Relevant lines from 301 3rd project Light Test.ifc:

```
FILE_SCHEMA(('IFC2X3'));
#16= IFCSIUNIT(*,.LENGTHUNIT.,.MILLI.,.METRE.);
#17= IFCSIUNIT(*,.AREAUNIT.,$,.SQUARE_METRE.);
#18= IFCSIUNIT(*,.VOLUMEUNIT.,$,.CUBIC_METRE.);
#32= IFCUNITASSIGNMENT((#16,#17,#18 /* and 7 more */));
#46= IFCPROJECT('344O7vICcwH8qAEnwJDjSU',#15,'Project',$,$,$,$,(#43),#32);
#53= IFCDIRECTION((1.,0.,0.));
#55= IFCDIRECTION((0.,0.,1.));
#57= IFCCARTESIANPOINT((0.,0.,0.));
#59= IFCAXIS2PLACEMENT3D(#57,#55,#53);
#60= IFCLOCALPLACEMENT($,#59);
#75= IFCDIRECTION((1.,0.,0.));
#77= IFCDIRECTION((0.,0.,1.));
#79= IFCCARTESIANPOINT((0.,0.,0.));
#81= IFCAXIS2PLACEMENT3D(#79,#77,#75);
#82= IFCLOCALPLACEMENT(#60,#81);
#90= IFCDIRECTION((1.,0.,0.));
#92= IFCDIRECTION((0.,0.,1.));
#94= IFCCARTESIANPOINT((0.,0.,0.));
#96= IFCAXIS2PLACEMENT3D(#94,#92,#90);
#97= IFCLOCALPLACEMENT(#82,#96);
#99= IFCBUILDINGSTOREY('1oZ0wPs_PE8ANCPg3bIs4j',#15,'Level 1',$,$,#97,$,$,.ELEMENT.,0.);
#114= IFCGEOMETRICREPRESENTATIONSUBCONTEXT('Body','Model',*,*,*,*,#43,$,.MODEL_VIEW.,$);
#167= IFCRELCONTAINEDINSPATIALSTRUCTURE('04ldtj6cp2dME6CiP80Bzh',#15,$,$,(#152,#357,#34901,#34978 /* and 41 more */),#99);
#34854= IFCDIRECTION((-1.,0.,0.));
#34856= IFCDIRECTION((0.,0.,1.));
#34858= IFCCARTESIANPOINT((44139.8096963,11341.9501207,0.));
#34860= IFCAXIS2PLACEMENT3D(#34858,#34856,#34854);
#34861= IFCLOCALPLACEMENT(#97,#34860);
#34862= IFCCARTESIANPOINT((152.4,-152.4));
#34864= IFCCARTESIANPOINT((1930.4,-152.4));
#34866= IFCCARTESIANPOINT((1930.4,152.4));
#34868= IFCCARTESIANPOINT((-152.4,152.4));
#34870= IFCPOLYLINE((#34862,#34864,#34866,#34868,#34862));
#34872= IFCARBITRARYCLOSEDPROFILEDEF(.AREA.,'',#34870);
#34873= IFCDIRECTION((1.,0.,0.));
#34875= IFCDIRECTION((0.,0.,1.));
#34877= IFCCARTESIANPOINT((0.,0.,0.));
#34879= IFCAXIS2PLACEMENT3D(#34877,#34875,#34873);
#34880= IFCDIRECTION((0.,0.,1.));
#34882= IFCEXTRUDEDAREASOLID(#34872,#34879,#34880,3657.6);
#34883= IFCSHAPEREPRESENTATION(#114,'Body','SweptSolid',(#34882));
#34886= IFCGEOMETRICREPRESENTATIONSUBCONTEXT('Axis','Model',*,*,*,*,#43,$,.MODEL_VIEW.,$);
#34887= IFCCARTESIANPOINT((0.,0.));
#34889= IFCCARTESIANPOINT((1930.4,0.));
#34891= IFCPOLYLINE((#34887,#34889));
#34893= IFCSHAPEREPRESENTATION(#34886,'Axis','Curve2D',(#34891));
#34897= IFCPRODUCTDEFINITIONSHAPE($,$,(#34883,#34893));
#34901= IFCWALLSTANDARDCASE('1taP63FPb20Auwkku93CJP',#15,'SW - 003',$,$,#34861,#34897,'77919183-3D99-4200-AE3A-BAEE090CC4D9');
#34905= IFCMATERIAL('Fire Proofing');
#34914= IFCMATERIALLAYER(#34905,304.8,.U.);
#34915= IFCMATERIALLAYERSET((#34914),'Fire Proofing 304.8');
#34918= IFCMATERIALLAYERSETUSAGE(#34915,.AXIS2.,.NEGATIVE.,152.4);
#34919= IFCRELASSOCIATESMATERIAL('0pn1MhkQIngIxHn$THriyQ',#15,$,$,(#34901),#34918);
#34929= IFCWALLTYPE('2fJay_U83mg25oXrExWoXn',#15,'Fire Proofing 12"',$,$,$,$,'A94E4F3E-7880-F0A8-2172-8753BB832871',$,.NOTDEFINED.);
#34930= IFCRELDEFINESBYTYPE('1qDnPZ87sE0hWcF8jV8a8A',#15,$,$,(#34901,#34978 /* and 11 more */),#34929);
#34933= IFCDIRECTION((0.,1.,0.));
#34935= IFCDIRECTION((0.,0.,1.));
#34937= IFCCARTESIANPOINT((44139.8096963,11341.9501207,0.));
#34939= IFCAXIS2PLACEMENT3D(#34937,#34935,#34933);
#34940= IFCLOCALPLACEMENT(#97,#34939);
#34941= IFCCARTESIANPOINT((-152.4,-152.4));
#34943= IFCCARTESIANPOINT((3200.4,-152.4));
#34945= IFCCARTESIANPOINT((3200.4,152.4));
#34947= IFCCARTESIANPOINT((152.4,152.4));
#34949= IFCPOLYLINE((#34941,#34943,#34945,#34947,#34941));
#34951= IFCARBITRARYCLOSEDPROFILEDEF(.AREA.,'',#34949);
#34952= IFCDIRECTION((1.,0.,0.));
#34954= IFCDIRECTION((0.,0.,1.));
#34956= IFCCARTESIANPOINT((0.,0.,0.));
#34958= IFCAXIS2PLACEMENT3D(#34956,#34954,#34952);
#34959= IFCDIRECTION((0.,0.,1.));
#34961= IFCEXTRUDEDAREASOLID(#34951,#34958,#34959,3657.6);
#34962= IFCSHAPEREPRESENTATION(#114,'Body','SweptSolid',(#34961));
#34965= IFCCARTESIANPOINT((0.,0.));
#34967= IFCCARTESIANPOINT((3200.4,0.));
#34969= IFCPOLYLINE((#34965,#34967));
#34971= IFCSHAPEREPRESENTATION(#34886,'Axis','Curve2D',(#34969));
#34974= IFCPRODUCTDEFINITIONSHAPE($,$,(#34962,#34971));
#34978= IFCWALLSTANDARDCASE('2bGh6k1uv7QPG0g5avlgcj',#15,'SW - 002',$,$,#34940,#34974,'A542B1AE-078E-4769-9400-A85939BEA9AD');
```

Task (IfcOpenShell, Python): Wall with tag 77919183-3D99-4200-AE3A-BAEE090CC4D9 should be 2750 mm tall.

```python
import ifcopenshell
import ifcopenshell.geom
import ifcopenshell.util.representation
import ifcopenshell.util.shape

model = ifcopenshell.open("301 3rd project Light Test.ifc")
settings = ifcopenshell.geom.settings()


def volume(element):
    """Net volume in cubic metres, openings subtracted."""
    shape = ifcopenshell.geom.create_shape(settings, element)
    return ifcopenshell.util.shape.get_volume(shape.geometry)


wall = model.by_guid("1taP63FPb20Auwkku93CJP")
before = volume(wall)

body = ifcopenshell.util.representation.get_representation(wall, "Model", "Body")
solid = body.Items[0]
old_height = solid.Depth
solid.Depth = 2750.0
after = volume(wall)

print(f"height {old_height:g} -> {solid.Depth:g}, volume {before:.3f} -> {after:.3f} m3")

model.write("301 3rd project Light Test_v2.ifc")
```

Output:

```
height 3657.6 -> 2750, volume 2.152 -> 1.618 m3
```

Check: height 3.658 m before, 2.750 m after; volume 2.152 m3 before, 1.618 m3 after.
